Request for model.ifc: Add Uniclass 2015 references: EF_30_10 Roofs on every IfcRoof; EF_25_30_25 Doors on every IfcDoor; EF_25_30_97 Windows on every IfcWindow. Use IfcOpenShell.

First a look at what the model holds.

```python
import ifcopenshell

model = ifcopenshell.open("model.ifc")
print(model.schema)
print("classifications:", [c.Name for c in model.by_type("IfcClassification")])
for ifc_class in ("IfcDoor", "IfcRoof", "IfcStair", "IfcWall", "IfcWindow"):
    print(ifc_class, len(model.by_type(ifc_class)))
```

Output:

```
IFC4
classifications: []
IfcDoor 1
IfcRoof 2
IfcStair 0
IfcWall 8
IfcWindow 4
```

```python
import ifcopenshell
import ifcopenshell.api.classification

model = ifcopenshell.open("model.ifc")

system = ifcopenshell.api.classification.add_classification(model, classification="Uniclass 2015")

codes = {
    "IfcRoof": ("EF_30_10", "Roofs"),
    "IfcDoor": ("EF_25_30_25", "Doors"),
    "IfcWindow": ("EF_25_30_97", "Windows"),
}
for ifc_class, (code, name) in codes.items():
    products = model.by_type(ifc_class)
    ifcopenshell.api.classification.add_reference(
        model, products=products, classification=system, identification=code, name=name
    )
    print(code, len(products))

model.write("model_v2.ifc")
```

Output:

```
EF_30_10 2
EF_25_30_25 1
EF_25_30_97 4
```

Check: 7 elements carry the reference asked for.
